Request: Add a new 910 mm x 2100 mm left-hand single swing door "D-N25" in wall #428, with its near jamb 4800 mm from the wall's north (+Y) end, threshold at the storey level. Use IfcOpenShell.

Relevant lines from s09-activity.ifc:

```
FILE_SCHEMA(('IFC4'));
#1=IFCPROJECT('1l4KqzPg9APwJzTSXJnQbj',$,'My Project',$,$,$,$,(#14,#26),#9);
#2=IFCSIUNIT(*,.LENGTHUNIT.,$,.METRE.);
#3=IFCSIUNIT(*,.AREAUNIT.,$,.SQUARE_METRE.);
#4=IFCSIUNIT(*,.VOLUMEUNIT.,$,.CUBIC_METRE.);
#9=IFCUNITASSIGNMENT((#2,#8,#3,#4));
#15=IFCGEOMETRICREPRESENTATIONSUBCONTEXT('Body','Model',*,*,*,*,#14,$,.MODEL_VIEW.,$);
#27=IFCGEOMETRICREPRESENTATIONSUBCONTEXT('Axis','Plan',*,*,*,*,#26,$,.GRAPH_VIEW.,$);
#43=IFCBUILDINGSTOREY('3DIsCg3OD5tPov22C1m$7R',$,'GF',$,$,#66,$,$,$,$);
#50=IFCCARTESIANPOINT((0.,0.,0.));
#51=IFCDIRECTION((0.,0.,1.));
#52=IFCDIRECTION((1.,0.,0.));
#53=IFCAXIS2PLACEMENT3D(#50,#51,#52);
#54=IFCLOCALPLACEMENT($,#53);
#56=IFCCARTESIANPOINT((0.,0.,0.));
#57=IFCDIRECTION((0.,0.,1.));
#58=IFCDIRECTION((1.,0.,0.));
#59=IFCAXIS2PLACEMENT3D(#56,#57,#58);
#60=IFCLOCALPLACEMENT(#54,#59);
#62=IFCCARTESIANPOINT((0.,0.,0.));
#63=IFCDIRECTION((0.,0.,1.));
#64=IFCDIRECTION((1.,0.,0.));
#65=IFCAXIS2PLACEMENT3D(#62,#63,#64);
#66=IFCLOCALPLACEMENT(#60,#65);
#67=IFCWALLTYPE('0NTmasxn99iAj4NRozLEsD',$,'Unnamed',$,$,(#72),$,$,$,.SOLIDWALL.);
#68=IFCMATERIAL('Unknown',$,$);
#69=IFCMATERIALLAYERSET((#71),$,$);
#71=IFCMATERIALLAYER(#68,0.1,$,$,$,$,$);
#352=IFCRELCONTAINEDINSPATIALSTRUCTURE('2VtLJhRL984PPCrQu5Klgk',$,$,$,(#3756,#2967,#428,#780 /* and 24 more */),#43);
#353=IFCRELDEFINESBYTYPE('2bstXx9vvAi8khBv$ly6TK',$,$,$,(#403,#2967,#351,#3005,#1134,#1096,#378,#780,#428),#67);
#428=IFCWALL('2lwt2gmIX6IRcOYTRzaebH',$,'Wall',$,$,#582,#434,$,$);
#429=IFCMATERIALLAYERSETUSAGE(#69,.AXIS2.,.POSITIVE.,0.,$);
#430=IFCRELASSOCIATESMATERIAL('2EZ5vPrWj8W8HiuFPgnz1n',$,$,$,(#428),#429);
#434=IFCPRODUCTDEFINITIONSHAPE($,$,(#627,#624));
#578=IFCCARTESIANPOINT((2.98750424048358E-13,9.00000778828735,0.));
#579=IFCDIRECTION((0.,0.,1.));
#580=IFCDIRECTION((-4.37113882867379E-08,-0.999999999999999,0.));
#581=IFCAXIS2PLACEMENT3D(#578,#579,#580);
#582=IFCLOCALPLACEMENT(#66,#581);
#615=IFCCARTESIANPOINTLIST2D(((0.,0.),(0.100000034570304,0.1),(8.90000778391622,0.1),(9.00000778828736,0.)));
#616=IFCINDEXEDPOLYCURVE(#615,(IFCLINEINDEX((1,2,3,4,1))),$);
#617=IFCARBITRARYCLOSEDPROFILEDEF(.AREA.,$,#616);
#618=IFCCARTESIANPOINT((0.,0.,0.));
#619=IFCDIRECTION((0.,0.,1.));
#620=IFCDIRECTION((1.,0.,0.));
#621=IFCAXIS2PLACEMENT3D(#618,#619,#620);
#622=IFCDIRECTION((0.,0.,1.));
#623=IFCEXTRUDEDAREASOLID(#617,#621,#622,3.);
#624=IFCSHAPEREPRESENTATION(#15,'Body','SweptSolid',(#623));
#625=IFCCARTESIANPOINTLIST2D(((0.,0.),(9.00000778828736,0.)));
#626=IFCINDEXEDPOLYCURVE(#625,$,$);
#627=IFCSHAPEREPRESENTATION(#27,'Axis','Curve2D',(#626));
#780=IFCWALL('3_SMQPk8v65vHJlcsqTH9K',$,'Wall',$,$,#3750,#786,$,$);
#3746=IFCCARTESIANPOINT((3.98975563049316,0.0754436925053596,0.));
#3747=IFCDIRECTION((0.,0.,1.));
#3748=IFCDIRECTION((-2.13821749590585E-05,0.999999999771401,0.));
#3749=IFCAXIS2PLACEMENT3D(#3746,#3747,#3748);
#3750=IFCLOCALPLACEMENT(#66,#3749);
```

```python
import numpy as np
import ifcopenshell
import ifcopenshell.api.feature
import ifcopenshell.api.geometry
import ifcopenshell.api.root
import ifcopenshell.api.spatial
import ifcopenshell.geom
import ifcopenshell.util.element
import ifcopenshell.util.placement
import ifcopenshell.util.representation
import ifcopenshell.util.shape
import ifcopenshell.util.unit

model = ifcopenshell.open("s09-activity.ifc")
unit_scale = ifcopenshell.util.unit.calculate_unit_scale(model)
settings = ifcopenshell.geom.settings()


def volume(element):
    """Net volume in cubic metres, openings subtracted."""
    shape = ifcopenshell.geom.create_shape(settings, element)
    return ifcopenshell.util.shape.get_volume(shape.geometry)


wall = model.by_guid("2lwt2gmIX6IRcOYTRzaebH")
storey = ifcopenshell.util.element.get_container(wall, ifc_class="IfcBuildingStorey")
context = ifcopenshell.util.representation.get_context(model, "Model", "Body", "MODEL_VIEW")
before = volume(wall)

width, height, from_end, sill = 0.91, 2.1, 4.8, 0.0  # metres

# The wall runs along its own X axis, and the end named is its -X end.
wall_shape = ifcopenshell.geom.create_shape(settings, wall)
x, y, z = ifcopenshell.util.shape.get_vertices(wall_shape.geometry).T
start = x.min() + from_end
face, thickness = float(y.min()), float(y.max() - y.min())
wall_matrix = ifcopenshell.util.placement.get_local_placement(wall.ObjectPlacement)
level = ifcopenshell.util.placement.get_local_placement(storey.ObjectPlacement)[2, 3]


def in_wall(x, y):
    """Placement at x, y metres in the wall's axes, at sill height."""
    matrix = wall_matrix.copy()
    matrix[:, 3] = wall_matrix @ np.array([x / unit_scale, y / unit_scale, 0.0, 1.0])
    matrix[2, 3] = level + sill / unit_scale
    return matrix


# Opening: a box that overshoots both wall faces by 50 mm.
opening = ifcopenshell.api.root.create_entity(model, ifc_class="IfcOpeningElement", predefined_type="OPENING")
box = ifcopenshell.api.geometry.add_wall_representation(
    model, context=context, length=width, height=height, thickness=thickness + 0.1
)
ifcopenshell.api.geometry.assign_representation(model, product=opening, representation=box)
ifcopenshell.api.geometry.edit_object_placement(model, product=opening, matrix=in_wall(start, face - 0.05), is_si=False)
ifcopenshell.api.feature.add_feature(model, feature=opening, element=wall)

door = ifcopenshell.api.root.create_entity(model, ifc_class="IfcDoor", name="D-N25", predefined_type="DOOR")
door.OverallWidth, door.OverallHeight = width / unit_scale, height / unit_scale
door.OperationType = "SINGLE_SWING_LEFT"
body = ifcopenshell.api.geometry.add_door_representation(
    model,
    context=context,
    overall_width=door.OverallWidth,
    overall_height=door.OverallHeight,
    operation_type="SINGLE_SWING_LEFT",
    lining_properties={"LiningDepth": thickness / unit_scale, "ThresholdDepth": thickness / unit_scale},
)
ifcopenshell.api.geometry.assign_representation(model, product=door, representation=body)
ifcopenshell.api.spatial.assign_container(model, products=[door], relating_structure=storey)
ifcopenshell.api.feature.add_filling(model, opening=opening, element=door)

# The lining spans the wall, so the door starts at the wall face.
ifcopenshell.api.geometry.edit_object_placement(model, product=door, matrix=in_wall(start, face), is_si=False)

after = volume(wall)

print(f"wall volume {before:.3f} -> {after:.3f} m3")

model.write("s09-activity-out.ifc")
```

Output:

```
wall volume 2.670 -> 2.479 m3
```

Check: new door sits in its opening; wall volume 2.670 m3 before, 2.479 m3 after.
